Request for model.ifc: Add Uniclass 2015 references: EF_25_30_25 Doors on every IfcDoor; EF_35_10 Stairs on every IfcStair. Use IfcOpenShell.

First a look at what the model holds.

```python
import ifcopenshell

model = ifcopenshell.open("model.ifc")
print(model.schema)
print("classifications:", [c.Name for c in model.by_type("IfcClassification")])
for ifc_class in ("IfcDoor", "IfcRoof", "IfcStair", "IfcWall", "IfcWindow"):
    print(ifc_class, len(model.by_type(ifc_class)))
```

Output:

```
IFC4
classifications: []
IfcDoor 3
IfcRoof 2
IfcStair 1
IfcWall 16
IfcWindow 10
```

```python
import ifcopenshell
import ifcopenshell.api.classification

model = ifcopenshell.open("model.ifc")

system = ifcopenshell.api.classification.add_classification(model, classification="Uniclass 2015")

codes = {
    "IfcDoor": ("EF_25_30_25", "Doors"),
    "IfcStair": ("EF_35_10", "Stairs"),
}
for ifc_class, (code, name) in codes.items():
    products = model.by_type(ifc_class)
    ifcopenshell.api.classification.add_reference(
        model, products=products, classification=system, identification=code, name=name
    )
    print(code, len(products))

model.write("model_edited.ifc")
```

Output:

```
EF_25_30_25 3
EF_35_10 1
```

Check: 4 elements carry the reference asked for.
